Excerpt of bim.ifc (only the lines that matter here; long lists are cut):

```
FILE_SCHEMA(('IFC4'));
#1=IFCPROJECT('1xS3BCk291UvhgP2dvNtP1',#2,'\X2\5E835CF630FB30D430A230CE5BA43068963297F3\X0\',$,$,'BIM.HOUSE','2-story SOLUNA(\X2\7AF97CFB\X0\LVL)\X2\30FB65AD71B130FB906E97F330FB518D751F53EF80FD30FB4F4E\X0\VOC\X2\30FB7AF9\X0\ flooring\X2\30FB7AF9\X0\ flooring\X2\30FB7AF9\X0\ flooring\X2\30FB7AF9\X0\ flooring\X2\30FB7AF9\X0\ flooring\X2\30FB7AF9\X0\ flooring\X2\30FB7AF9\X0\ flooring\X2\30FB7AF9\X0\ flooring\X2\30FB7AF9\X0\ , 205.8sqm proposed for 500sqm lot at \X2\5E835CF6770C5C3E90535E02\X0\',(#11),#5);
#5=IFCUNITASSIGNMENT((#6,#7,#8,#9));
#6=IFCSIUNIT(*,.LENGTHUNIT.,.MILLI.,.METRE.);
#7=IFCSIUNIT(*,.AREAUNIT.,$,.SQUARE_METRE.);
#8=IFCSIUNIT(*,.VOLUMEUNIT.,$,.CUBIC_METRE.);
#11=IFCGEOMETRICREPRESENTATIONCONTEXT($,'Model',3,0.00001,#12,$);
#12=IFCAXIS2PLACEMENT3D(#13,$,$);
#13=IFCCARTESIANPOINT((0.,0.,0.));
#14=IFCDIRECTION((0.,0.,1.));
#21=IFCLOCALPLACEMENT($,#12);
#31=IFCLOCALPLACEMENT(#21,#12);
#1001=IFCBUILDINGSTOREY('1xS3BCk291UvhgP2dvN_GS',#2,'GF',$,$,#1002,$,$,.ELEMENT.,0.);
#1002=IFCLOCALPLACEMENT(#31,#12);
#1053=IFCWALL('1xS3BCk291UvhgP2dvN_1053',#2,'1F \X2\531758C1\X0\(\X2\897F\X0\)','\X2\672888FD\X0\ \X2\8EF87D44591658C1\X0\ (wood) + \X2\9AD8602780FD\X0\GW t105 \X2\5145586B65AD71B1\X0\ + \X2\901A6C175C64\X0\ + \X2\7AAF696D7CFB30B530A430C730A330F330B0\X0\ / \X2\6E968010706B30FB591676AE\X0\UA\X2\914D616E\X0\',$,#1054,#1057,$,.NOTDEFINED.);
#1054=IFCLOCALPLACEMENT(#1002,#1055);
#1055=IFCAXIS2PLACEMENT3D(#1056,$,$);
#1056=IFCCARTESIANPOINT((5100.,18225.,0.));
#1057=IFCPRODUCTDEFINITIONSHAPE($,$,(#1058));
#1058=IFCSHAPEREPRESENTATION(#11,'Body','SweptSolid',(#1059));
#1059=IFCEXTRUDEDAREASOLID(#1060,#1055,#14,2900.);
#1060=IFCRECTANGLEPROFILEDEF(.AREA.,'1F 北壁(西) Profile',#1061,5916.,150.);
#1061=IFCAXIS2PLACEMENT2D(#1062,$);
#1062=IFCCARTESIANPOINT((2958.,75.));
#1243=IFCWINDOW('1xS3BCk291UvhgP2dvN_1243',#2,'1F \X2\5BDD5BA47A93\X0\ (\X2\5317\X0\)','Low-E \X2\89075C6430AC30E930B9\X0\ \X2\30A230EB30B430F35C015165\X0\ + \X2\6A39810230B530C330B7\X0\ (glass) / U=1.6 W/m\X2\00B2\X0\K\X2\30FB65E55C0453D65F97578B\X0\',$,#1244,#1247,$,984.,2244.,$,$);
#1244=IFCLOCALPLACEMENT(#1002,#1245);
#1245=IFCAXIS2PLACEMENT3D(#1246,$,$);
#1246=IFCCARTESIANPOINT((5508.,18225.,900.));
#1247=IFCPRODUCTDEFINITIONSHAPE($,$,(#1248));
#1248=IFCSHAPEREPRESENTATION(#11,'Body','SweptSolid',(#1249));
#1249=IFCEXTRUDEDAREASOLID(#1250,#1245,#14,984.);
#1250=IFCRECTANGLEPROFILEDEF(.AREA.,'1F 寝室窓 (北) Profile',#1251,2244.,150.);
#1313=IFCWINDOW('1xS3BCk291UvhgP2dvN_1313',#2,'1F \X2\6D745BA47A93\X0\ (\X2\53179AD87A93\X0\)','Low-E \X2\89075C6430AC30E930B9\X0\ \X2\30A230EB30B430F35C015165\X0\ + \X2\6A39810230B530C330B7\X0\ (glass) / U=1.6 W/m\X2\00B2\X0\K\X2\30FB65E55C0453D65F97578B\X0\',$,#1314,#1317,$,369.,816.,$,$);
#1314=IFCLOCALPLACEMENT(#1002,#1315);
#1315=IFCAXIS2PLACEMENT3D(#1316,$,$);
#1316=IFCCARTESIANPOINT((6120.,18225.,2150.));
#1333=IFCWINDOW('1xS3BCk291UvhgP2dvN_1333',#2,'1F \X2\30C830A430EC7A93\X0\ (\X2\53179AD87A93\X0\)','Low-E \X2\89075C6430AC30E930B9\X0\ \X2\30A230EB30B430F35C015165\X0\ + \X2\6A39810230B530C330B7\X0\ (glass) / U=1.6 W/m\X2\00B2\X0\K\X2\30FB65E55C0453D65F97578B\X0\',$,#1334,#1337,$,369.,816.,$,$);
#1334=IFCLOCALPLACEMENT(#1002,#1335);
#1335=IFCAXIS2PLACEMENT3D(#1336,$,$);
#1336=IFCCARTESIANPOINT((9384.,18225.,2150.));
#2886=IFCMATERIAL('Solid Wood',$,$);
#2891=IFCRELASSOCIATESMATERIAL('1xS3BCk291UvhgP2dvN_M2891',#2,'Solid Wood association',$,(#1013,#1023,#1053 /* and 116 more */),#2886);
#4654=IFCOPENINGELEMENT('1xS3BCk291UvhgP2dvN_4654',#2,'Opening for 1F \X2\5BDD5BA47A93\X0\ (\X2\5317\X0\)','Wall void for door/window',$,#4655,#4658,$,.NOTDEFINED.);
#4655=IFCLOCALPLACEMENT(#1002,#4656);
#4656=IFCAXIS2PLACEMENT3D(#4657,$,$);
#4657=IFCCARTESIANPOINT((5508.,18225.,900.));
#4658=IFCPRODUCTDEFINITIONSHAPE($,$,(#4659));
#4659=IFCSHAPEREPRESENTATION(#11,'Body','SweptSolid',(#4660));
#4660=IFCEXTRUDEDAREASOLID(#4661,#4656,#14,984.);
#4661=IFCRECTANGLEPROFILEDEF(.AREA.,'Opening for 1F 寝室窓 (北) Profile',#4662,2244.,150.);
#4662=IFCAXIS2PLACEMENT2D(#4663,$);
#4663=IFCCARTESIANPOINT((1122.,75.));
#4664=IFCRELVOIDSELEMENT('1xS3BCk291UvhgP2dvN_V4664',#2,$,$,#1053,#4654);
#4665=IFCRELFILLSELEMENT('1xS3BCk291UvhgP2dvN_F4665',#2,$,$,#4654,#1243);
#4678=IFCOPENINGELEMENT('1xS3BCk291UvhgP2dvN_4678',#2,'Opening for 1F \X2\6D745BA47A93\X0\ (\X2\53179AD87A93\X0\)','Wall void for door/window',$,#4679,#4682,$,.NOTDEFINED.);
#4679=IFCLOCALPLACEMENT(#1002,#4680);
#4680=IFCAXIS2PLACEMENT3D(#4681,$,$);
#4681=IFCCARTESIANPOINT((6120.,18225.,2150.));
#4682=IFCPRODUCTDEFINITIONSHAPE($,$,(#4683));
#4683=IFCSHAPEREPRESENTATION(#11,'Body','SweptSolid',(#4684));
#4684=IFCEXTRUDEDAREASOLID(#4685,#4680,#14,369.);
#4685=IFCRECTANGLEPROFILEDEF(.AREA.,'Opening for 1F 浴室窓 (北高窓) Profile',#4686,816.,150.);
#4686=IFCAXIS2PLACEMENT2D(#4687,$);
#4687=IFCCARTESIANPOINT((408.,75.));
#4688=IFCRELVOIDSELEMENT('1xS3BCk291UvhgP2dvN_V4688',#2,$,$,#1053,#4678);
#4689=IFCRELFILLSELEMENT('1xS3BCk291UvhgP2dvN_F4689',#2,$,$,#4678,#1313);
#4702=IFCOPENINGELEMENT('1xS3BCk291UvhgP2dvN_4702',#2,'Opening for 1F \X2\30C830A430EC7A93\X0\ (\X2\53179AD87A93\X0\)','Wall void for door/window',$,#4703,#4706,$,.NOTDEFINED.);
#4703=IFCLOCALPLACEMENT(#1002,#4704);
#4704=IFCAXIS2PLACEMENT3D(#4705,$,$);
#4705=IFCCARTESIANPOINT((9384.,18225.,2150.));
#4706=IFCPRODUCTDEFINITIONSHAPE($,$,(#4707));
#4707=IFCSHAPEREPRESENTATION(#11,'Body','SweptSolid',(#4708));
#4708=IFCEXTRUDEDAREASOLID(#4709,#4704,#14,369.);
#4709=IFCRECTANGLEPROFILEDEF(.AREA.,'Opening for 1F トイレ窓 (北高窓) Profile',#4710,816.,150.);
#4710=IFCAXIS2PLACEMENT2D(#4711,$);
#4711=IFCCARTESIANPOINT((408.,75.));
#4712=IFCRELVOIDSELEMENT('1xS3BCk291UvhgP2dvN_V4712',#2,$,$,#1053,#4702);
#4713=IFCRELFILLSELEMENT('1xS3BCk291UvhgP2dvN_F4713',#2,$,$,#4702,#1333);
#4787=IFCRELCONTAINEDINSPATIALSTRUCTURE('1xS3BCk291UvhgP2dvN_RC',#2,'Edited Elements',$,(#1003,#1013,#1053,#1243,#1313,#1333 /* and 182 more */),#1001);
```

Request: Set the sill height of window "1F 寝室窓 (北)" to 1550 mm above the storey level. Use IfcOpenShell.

```python
import numpy as np
import ifcopenshell
import ifcopenshell.api.geometry
import ifcopenshell.geom
import ifcopenshell.util.element
import ifcopenshell.util.placement
import ifcopenshell.util.shape
import ifcopenshell.util.unit

model = ifcopenshell.open("bim.ifc")
unit_scale = ifcopenshell.util.unit.calculate_unit_scale(model)

window = model.by_guid("1xS3BCk291UvhgP2dvN_1243")
opening = window.FillsVoids[0].RelatingOpeningElement
storey = ifcopenshell.util.element.get_container(window, ifc_class="IfcBuildingStorey")
level = ifcopenshell.util.placement.get_local_placement(storey.ObjectPlacement)[2, 3]

# The opening's origin need not be at the sill, so measure its lowest point.
shape = ifcopenshell.geom.create_shape(ifcopenshell.geom.settings(), opening)
bottom = ifcopenshell.util.shape.get_shape_bottom_elevation(shape, shape.geometry) / unit_scale
dz = level + 1.55 / unit_scale - bottom

shift = np.array([0.0, 0.0, dz])
# The window is not placed relative to its opening, so move both.
for product in (opening, window):
    matrix = ifcopenshell.util.placement.get_local_placement(product.ObjectPlacement)
    matrix[:3, 3] += shift
    ifcopenshell.api.geometry.edit_object_placement(model, product=product, matrix=matrix, is_si=False)

print(f"moved by {dz * unit_scale:+.3f} m")

model.write("bim_rev.ifc")
```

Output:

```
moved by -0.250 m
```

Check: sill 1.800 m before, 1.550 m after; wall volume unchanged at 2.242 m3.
